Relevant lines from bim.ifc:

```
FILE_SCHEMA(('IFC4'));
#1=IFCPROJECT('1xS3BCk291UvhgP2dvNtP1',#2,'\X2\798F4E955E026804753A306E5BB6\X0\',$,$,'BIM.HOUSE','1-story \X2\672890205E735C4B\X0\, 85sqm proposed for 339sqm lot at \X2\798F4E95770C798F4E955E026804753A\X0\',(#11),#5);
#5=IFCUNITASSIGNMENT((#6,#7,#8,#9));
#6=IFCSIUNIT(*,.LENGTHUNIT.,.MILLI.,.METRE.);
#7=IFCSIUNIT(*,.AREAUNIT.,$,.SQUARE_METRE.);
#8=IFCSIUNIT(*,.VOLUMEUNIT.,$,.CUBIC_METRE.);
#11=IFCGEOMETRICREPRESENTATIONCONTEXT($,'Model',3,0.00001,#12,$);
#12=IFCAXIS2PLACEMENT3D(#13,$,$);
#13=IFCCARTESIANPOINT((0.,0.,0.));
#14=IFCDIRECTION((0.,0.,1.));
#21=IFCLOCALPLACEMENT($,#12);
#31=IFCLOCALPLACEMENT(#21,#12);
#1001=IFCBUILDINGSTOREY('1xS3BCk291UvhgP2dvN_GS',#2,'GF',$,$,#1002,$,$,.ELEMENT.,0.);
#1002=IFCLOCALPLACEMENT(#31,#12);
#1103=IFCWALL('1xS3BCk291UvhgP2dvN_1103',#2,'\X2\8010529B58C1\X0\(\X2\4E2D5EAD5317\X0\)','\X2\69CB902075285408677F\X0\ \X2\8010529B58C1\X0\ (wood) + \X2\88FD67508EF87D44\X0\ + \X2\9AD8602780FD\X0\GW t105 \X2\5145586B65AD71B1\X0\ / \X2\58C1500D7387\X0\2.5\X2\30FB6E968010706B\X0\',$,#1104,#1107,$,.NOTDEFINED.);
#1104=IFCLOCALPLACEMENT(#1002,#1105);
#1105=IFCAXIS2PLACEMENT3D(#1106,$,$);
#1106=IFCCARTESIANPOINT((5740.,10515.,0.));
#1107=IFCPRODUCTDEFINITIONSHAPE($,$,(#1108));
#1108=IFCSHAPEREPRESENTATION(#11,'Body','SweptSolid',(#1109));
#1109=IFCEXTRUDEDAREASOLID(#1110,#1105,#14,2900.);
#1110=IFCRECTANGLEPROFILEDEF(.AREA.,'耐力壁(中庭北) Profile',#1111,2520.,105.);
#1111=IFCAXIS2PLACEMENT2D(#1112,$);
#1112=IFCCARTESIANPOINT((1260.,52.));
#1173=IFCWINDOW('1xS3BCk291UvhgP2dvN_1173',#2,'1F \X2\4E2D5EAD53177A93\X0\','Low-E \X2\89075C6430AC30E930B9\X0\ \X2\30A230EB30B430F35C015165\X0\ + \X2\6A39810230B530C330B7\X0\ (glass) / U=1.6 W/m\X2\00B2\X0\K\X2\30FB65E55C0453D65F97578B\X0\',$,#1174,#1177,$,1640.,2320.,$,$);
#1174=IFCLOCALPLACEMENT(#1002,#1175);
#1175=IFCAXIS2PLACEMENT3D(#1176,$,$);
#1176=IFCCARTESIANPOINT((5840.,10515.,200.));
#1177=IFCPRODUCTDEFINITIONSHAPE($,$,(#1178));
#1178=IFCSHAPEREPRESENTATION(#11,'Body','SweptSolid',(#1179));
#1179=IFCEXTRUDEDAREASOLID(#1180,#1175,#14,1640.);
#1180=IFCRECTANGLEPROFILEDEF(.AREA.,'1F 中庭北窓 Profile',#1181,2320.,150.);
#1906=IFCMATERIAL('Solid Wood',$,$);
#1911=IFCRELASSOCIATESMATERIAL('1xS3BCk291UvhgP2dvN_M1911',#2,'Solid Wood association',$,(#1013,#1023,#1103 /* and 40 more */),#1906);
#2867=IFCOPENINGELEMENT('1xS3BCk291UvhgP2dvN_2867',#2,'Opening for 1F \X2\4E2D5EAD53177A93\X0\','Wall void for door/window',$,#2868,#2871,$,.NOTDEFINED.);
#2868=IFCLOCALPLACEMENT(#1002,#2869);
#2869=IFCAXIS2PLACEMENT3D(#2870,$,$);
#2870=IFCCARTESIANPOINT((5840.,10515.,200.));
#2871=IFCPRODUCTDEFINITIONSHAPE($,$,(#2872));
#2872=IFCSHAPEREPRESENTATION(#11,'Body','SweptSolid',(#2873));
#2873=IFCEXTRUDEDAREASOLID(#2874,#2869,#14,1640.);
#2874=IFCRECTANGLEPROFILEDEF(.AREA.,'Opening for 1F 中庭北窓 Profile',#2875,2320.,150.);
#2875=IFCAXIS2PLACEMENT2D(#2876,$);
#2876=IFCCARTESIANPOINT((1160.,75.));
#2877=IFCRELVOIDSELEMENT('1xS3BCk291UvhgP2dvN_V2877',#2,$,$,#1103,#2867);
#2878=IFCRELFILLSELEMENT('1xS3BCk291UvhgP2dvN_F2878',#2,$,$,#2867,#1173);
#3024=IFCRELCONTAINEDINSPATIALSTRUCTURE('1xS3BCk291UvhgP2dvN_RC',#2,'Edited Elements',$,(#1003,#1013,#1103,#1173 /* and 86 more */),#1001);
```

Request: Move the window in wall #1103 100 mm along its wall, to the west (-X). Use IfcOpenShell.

```python
import ifcopenshell
import ifcopenshell.api.geometry
import ifcopenshell.util.placement

model = ifcopenshell.open("bim.ifc")

window = model.by_guid("1xS3BCk291UvhgP2dvN_1173")
opening = window.FillsVoids[0].RelatingOpeningElement
wall = opening.VoidsElements[0].RelatingBuildingElement

wall_matrix = ifcopenshell.util.placement.get_local_placement(wall.ObjectPlacement)
shift = wall_matrix[:3, 0] * -100.0
before = ifcopenshell.util.placement.get_local_placement(window.ObjectPlacement)[:3, 3].copy()

# The window is not placed relative to its opening, so move both.
for product in (opening, window):
    matrix = ifcopenshell.util.placement.get_local_placement(product.ObjectPlacement)
    matrix[:3, 3] += shift
    ifcopenshell.api.geometry.edit_object_placement(model, product=product, matrix=matrix, is_si=False)

after = ifcopenshell.util.placement.get_local_placement(window.ObjectPlacement)[:3, 3]
print("window moved by", (after - before).round(3) + 0.0)

model.write("bim_edited.ifc")
```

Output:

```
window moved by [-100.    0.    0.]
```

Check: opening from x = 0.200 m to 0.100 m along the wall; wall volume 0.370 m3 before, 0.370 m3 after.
